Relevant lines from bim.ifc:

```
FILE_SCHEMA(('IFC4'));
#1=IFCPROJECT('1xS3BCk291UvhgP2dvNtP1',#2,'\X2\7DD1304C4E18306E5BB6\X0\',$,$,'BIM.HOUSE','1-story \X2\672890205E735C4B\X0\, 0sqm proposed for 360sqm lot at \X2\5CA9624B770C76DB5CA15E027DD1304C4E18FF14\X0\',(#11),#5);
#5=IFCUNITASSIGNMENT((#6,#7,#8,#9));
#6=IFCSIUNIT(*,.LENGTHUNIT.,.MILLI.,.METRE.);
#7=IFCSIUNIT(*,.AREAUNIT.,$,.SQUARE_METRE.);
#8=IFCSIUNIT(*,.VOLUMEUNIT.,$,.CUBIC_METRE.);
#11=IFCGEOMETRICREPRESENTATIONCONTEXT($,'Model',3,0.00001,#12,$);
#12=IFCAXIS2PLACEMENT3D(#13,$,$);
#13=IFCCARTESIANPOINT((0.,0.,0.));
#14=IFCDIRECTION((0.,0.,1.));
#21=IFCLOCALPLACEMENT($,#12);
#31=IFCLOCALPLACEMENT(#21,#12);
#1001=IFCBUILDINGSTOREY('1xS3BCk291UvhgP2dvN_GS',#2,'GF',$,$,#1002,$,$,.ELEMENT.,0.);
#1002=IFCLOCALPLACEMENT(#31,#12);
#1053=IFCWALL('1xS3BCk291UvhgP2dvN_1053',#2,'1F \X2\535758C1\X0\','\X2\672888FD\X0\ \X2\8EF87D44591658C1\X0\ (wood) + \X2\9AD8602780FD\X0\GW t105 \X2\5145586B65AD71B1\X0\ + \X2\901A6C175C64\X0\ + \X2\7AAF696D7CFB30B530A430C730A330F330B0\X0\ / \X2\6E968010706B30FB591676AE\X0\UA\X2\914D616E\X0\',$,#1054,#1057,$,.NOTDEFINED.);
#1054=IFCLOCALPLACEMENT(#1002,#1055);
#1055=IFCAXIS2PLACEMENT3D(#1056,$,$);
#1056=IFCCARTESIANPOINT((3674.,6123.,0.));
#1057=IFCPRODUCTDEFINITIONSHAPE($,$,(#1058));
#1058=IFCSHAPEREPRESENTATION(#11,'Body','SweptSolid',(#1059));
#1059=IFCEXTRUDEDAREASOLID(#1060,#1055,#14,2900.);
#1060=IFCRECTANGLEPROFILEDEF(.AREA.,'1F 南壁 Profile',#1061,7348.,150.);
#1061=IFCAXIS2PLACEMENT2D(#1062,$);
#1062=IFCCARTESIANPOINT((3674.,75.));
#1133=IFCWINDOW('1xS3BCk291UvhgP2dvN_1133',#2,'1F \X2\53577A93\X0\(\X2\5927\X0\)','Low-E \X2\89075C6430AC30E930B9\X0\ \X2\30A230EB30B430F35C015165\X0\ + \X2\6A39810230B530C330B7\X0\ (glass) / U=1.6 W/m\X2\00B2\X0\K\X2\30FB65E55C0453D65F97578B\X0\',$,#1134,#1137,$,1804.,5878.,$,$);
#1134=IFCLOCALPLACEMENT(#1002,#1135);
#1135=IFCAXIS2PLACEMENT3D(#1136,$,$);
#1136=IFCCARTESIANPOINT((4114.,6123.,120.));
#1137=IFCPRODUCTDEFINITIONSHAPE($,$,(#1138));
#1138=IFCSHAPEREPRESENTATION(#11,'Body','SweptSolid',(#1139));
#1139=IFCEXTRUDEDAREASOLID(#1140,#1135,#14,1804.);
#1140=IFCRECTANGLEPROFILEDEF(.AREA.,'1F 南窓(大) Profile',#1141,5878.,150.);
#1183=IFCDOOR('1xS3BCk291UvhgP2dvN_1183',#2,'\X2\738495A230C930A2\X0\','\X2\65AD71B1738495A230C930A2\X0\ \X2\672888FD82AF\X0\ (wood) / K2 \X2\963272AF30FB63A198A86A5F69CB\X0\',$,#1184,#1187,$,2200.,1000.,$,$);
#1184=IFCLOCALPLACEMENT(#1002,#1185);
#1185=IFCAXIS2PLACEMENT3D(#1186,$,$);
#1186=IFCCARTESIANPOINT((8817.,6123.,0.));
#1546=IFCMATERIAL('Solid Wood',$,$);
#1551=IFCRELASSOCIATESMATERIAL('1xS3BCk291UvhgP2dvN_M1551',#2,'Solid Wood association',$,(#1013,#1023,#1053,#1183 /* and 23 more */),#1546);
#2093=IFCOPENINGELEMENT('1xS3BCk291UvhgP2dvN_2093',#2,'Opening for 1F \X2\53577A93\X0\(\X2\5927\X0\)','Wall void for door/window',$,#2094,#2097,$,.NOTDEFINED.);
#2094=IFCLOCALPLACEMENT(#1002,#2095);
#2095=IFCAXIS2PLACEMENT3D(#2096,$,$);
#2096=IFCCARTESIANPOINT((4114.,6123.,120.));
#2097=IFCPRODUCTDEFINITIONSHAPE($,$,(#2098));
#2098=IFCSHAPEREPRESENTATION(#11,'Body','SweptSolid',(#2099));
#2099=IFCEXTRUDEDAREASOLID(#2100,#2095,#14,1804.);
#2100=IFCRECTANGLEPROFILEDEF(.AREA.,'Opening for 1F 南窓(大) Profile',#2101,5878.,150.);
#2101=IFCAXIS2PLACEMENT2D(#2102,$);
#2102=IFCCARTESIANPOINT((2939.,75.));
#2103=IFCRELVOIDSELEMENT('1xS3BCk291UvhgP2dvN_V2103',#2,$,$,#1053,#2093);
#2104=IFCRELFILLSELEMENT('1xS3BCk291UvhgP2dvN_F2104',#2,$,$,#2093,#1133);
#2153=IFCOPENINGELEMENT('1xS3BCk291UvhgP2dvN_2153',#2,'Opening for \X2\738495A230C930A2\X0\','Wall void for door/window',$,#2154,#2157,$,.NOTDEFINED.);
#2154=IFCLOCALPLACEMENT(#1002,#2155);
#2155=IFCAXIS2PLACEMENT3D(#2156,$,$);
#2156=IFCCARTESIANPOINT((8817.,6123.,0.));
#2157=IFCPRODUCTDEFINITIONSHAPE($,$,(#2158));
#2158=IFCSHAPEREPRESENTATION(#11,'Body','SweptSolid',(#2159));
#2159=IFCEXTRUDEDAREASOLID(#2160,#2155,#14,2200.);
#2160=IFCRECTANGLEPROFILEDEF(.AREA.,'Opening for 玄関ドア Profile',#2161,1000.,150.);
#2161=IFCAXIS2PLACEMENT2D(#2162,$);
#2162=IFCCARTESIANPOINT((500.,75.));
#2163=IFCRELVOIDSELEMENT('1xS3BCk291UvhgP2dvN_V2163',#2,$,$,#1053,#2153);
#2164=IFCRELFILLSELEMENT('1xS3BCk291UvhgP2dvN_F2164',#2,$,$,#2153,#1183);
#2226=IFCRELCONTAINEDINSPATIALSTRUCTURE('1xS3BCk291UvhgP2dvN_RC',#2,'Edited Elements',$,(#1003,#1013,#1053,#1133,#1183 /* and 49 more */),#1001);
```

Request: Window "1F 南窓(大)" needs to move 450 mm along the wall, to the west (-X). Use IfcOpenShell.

```python
import ifcopenshell
import ifcopenshell.api.geometry
import ifcopenshell.util.placement
import ifcopenshell.util.unit

model = ifcopenshell.open("bim.ifc")
unit_scale = ifcopenshell.util.unit.calculate_unit_scale(model)

window = model.by_id(1133)
opening = window.FillsVoids[0].RelatingOpeningElement
wall = opening.VoidsElements[0].RelatingBuildingElement

wall_matrix = ifcopenshell.util.placement.get_local_placement(wall.ObjectPlacement)
shift = wall_matrix[:3, 0] * -0.45 / unit_scale
before = ifcopenshell.util.placement.get_local_placement(window.ObjectPlacement)[:3, 3].copy()

# The window is not placed relative to its opening, so move both.
for product in (opening, window):
    matrix = ifcopenshell.util.placement.get_local_placement(product.ObjectPlacement)
    matrix[:3, 3] += shift
    ifcopenshell.api.geometry.edit_object_placement(model, product=product, matrix=matrix, is_si=False)

after = ifcopenshell.util.placement.get_local_placement(window.ObjectPlacement)[:3, 3]
print("window moved by", (after - before).round(3) + 0.0)

model.write("bim_updated.ifc")
```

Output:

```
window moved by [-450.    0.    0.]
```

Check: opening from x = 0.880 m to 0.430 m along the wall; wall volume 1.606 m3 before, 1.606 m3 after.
